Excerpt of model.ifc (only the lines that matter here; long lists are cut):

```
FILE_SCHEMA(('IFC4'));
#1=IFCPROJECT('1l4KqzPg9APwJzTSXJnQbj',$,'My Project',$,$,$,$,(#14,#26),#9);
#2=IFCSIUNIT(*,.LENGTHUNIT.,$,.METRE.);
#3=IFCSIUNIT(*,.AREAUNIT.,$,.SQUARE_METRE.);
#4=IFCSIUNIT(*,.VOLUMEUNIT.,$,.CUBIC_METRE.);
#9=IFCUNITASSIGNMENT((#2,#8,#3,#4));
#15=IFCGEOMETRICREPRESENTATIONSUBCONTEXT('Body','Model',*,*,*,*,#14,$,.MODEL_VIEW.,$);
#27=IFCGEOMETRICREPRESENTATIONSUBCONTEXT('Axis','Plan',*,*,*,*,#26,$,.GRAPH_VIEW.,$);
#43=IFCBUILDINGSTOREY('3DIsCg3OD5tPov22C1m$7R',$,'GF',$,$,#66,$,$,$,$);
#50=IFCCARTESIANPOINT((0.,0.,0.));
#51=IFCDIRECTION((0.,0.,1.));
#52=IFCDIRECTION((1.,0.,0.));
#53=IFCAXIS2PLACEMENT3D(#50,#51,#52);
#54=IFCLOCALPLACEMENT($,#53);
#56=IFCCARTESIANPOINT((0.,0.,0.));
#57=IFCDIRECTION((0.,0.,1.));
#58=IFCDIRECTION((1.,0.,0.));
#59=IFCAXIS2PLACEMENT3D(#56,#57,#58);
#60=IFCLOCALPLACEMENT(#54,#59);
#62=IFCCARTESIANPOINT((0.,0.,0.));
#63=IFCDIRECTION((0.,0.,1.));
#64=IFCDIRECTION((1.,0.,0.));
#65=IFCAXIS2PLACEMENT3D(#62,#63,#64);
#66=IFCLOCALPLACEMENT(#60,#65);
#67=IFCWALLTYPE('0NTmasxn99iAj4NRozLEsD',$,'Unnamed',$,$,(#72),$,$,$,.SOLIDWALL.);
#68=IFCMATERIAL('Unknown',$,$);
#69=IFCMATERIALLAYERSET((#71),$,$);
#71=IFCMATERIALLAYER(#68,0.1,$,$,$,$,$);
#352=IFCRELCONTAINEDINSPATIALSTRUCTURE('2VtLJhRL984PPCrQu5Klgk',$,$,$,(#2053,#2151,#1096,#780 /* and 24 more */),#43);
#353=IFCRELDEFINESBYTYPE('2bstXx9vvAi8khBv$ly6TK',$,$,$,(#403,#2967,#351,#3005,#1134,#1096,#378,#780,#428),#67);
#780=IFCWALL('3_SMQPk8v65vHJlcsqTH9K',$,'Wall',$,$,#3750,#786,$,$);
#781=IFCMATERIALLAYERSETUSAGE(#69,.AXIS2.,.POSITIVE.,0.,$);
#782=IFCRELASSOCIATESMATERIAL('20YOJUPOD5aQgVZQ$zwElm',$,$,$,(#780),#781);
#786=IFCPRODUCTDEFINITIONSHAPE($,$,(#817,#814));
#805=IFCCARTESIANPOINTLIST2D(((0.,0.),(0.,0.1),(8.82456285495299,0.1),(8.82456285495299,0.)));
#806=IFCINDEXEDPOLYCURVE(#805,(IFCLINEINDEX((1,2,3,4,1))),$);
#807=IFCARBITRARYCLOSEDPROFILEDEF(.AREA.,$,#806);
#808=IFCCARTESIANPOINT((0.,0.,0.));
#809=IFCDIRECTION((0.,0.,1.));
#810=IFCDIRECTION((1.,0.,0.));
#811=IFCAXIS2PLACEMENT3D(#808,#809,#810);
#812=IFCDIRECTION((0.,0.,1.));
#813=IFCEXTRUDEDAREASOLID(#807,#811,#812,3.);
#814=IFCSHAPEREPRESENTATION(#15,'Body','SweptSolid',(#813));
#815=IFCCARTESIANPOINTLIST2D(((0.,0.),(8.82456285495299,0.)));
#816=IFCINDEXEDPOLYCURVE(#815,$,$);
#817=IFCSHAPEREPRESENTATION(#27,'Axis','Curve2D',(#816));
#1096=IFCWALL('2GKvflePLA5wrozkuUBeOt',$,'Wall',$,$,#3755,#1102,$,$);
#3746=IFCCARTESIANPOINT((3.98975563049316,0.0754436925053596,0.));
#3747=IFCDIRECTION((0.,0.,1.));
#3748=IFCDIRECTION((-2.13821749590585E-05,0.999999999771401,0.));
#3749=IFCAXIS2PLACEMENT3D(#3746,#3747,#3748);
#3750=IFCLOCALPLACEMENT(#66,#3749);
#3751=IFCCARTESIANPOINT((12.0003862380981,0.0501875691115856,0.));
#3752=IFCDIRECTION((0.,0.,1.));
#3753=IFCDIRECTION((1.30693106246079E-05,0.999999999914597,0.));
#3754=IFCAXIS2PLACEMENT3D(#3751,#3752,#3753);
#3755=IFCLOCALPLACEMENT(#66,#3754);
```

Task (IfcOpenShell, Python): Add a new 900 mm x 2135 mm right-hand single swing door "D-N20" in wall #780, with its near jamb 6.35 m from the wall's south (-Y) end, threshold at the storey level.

```python
import numpy as np
import ifcopenshell
import ifcopenshell.api.feature
import ifcopenshell.api.geometry
import ifcopenshell.api.root
import ifcopenshell.api.spatial
import ifcopenshell.geom
import ifcopenshell.util.element
import ifcopenshell.util.placement
import ifcopenshell.util.representation
import ifcopenshell.util.shape
import ifcopenshell.util.unit

model = ifcopenshell.open("model.ifc")
unit_scale = ifcopenshell.util.unit.calculate_unit_scale(model)
settings = ifcopenshell.geom.settings()


def volume(element):
    """Net volume in cubic metres, openings subtracted."""
    shape = ifcopenshell.geom.create_shape(settings, element)
    return ifcopenshell.util.shape.get_volume(shape.geometry)


wall = model.by_guid("3_SMQPk8v65vHJlcsqTH9K")
storey = ifcopenshell.util.element.get_container(wall, ifc_class="IfcBuildingStorey")
context = ifcopenshell.util.representation.get_context(model, "Model", "Body", "MODEL_VIEW")
before = volume(wall)

width, height, from_end, sill = 0.9, 2.135, 6.35, 0.0  # metres

# The wall runs along its own X axis, and the end named is its -X end.
wall_shape = ifcopenshell.geom.create_shape(settings, wall)
x, y, z = ifcopenshell.util.shape.get_vertices(wall_shape.geometry).T
start = x.min() + from_end
face, thickness = float(y.min()), float(y.max() - y.min())
wall_matrix = ifcopenshell.util.placement.get_local_placement(wall.ObjectPlacement)
level = ifcopenshell.util.placement.get_local_placement(storey.ObjectPlacement)[2, 3]


def in_wall(x, y):
    """Placement at x, y metres in the wall's axes, at sill height."""
    matrix = wall_matrix.copy()
    matrix[:, 3] = wall_matrix @ np.array([x / unit_scale, y / unit_scale, 0.0, 1.0])
    matrix[2, 3] = level + sill / unit_scale
    return matrix


# Opening: a box that overshoots both wall faces by 50 mm.
opening = ifcopenshell.api.root.create_entity(model, ifc_class="IfcOpeningElement", predefined_type="OPENING")
box = ifcopenshell.api.geometry.add_wall_representation(
    model, context=context, length=width, height=height, thickness=thickness + 0.1
)
ifcopenshell.api.geometry.assign_representation(model, product=opening, representation=box)
ifcopenshell.api.geometry.edit_object_placement(model, product=opening, matrix=in_wall(start, face - 0.05), is_si=False)
ifcopenshell.api.feature.add_feature(model, feature=opening, element=wall)

door = ifcopenshell.api.root.create_entity(model, ifc_class="IfcDoor", name="D-N20", predefined_type="DOOR")
door.OverallWidth, door.OverallHeight = width / unit_scale, height / unit_scale
door.OperationType = "SINGLE_SWING_RIGHT"
body = ifcopenshell.api.geometry.add_door_representation(
    model,
    context=context,
    overall_width=door.OverallWidth,
    overall_height=door.OverallHeight,
    operation_type="SINGLE_SWING_RIGHT",
    lining_properties={"LiningDepth": thickness / unit_scale, "ThresholdDepth": thickness / unit_scale},
)
ifcopenshell.api.geometry.assign_representation(model, product=door, representation=body)
ifcopenshell.api.spatial.assign_container(model, products=[door], relating_structure=storey)
ifcopenshell.api.feature.add_filling(model, opening=opening, element=door)

# The lining spans the wall, so the door starts at the wall face.
ifcopenshell.api.geometry.edit_object_placement(model, product=door, matrix=in_wall(start, face), is_si=False)

after = volume(wall)

print(f"wall volume {before:.3f} -> {after:.3f} m3")

model.write("model_rev.ifc")
```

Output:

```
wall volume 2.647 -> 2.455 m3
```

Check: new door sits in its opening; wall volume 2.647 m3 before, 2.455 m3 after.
